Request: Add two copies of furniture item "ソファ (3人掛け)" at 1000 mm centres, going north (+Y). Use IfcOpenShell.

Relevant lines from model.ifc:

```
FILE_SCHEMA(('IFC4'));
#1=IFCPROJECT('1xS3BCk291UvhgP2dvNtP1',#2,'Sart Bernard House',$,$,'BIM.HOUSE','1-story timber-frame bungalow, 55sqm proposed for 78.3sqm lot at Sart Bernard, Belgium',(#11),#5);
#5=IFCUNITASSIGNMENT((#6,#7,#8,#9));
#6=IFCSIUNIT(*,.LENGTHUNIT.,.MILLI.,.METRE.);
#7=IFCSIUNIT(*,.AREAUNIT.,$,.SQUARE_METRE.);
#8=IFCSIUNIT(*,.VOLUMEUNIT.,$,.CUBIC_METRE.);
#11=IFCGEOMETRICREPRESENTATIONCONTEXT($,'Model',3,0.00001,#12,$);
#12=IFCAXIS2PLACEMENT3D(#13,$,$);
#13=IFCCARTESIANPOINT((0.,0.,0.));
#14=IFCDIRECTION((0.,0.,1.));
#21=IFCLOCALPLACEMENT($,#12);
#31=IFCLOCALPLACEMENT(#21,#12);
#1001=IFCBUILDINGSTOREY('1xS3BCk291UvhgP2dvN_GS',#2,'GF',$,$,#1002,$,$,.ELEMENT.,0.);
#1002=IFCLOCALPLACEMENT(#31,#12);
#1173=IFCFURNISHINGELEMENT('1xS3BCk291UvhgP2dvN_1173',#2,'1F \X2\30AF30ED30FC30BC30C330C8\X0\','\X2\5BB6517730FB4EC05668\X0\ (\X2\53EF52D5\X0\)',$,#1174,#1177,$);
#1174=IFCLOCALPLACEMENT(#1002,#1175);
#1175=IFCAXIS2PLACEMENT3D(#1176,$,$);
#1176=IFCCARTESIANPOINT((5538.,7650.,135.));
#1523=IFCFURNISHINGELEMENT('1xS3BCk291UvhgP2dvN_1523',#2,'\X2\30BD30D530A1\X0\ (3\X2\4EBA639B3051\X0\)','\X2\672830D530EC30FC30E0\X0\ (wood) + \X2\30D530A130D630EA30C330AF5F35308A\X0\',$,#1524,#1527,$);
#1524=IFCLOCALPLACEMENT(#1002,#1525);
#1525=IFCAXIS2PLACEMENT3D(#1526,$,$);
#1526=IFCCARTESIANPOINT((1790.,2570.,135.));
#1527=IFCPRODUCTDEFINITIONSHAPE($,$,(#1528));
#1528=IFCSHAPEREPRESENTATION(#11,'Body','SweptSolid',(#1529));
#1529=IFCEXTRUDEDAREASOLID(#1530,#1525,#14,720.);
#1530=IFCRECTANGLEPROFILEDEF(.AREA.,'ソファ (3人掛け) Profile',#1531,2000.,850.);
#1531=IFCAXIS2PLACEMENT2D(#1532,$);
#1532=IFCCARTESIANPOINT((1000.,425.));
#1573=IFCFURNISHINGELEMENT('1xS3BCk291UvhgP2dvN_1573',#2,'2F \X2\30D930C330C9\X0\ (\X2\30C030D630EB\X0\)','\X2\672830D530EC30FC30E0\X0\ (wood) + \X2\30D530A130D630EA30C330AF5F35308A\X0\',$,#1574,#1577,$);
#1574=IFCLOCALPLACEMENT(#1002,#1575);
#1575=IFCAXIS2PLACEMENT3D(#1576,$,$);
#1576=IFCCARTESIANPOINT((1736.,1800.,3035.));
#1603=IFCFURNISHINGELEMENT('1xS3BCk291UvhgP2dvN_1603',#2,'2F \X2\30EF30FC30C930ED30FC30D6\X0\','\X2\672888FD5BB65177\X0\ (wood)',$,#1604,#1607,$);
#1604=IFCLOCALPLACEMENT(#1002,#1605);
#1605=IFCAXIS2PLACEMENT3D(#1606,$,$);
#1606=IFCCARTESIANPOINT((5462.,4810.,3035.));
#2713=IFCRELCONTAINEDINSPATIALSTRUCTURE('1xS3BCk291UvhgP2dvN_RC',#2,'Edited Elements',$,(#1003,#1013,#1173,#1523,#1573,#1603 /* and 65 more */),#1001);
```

```python
import numpy as np
import ifcopenshell
import ifcopenshell.api.geometry
import ifcopenshell.api.root
import ifcopenshell.util.element
import ifcopenshell.util.placement
import ifcopenshell.util.unit

model = ifcopenshell.open("model.ifc")
unit_scale = ifcopenshell.util.unit.calculate_unit_scale(model)


def reuse_history(source, copy):
    """copy_class also copies each property set's owner history, people and application; keep the originals."""
    for rel in copy.IsDefinedBy:
        if rel.is_a("IfcRelDefinesByProperties") and (history := rel.RelatingPropertyDefinition.OwnerHistory):
            rel.RelatingPropertyDefinition.OwnerHistory = source.OwnerHistory
            ifcopenshell.util.element.remove_deep2(model, history)


source = model.by_guid("1xS3BCk291UvhgP2dvN_1523")
base = ifcopenshell.util.placement.get_local_placement(source.ObjectPlacement)
step = np.array([0.0, 1.0, 0.0]) * 1 / unit_scale

for i in range(1, 3):
    copy = ifcopenshell.api.root.copy_class(model, product=source)
    copy.Representation = ifcopenshell.util.element.copy_deep(
        model, source.Representation, exclude=["IfcGeometricRepresentationContext", "IfcRepresentationMap"]
    )
    reuse_history(source, copy)
    matrix = base.copy()
    matrix[:3, 3] += i * step
    print("added at", matrix[:3, 3].round(3) + 0.0)
    ifcopenshell.api.geometry.edit_object_placement(model, product=copy, matrix=matrix, is_si=False)

model.write("model_edited.ifc")
```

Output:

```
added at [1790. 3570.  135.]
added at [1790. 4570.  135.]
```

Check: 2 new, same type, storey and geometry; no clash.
